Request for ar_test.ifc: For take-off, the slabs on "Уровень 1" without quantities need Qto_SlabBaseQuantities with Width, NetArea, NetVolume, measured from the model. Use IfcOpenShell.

First a look at what the model holds.

```python
import ifcopenshell
import ifcopenshell.util.element
import ifcopenshell.util.unit

model = ifcopenshell.open("ar_test.ifc")
print(model.schema)
for unit_type in ("LENGTHUNIT", "AREAUNIT", "VOLUMEUNIT"):
    print(unit_type, ifcopenshell.util.unit.calculate_unit_scale(model, unit_type))
storey = next(s for s in model.by_type("IfcBuildingStorey") if s.Name == "Уровень 1")
slabs = [e for e in ifcopenshell.util.element.get_decomposition(storey) if e.is_a("IfcSlab")]
for e in sorted(slabs, key=lambda e: e.id()):
    print(e.id(), e.is_a(), e.Name, list(ifcopenshell.util.element.get_psets(e, qtos_only=True)), sep=" | ")
```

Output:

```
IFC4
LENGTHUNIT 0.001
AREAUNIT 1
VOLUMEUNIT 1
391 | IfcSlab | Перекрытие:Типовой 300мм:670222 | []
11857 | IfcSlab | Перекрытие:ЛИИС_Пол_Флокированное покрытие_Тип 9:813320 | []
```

```python
import ifcopenshell
import ifcopenshell.api.pset
import ifcopenshell.geom
import ifcopenshell.util.element
import ifcopenshell.util.shape
import ifcopenshell.util.unit

model = ifcopenshell.open("ar_test.ifc")
unit_scale = ifcopenshell.util.unit.calculate_unit_scale(model)
area_scale = ifcopenshell.util.unit.calculate_unit_scale(model, "AREAUNIT")
volume_scale = ifcopenshell.util.unit.calculate_unit_scale(model, "VOLUMEUNIT")
settings = ifcopenshell.geom.settings()

storey = next(s for s in model.by_type("IfcBuildingStorey") if s.Name == "Уровень 1")
slabs = [e for e in ifcopenshell.util.element.get_decomposition(storey) if e.is_a("IfcSlab")]

for e in sorted(slabs, key=lambda e: e.id()):
    if ifcopenshell.util.element.get_psets(e, qtos_only=True, should_inherit=False):
        continue
    # Geometry comes back in metres, in the element's own axes.
    shape = ifcopenshell.geom.create_shape(settings, e)
    values = {
        "Width": ifcopenshell.util.shape.get_z(shape.geometry) / unit_scale,
        "NetArea": ifcopenshell.util.shape.get_footprint_area(shape.geometry) / area_scale,
        "NetVolume": ifcopenshell.util.shape.get_volume(shape.geometry) / volume_scale,
    }
    qto = ifcopenshell.api.pset.add_qto(model, product=e, name="Qto_SlabBaseQuantities")
    ifcopenshell.api.pset.edit_qto(model, qto=qto, properties=values)
    print(e.id(), {k: round(v, 3) for k, v in values.items()})

model.write("ar_test_edited.ifc")
```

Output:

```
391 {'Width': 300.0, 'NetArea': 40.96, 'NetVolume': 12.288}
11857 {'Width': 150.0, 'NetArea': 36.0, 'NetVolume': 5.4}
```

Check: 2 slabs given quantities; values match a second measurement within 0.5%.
